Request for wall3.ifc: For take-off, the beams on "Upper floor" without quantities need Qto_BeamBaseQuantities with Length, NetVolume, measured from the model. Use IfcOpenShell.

First a look at what the model holds.

```python
import ifcopenshell
import ifcopenshell.util.element
import ifcopenshell.util.unit

model = ifcopenshell.open("wall3.ifc")
print(model.schema)
for unit_type in ("LENGTHUNIT", "AREAUNIT", "VOLUMEUNIT"):
    print(unit_type, ifcopenshell.util.unit.calculate_unit_scale(model, unit_type))
storey = next(s for s in model.by_type("IfcBuildingStorey") if s.Name == "Upper floor")
beams = [e for e in ifcopenshell.util.element.get_decomposition(storey) if e.is_a("IfcBeam")]
for e in sorted(beams, key=lambda e: e.id()):
    print(e.id(), e.is_a(), e.Name, list(ifcopenshell.util.element.get_psets(e, qtos_only=True)), sep=" | ")
```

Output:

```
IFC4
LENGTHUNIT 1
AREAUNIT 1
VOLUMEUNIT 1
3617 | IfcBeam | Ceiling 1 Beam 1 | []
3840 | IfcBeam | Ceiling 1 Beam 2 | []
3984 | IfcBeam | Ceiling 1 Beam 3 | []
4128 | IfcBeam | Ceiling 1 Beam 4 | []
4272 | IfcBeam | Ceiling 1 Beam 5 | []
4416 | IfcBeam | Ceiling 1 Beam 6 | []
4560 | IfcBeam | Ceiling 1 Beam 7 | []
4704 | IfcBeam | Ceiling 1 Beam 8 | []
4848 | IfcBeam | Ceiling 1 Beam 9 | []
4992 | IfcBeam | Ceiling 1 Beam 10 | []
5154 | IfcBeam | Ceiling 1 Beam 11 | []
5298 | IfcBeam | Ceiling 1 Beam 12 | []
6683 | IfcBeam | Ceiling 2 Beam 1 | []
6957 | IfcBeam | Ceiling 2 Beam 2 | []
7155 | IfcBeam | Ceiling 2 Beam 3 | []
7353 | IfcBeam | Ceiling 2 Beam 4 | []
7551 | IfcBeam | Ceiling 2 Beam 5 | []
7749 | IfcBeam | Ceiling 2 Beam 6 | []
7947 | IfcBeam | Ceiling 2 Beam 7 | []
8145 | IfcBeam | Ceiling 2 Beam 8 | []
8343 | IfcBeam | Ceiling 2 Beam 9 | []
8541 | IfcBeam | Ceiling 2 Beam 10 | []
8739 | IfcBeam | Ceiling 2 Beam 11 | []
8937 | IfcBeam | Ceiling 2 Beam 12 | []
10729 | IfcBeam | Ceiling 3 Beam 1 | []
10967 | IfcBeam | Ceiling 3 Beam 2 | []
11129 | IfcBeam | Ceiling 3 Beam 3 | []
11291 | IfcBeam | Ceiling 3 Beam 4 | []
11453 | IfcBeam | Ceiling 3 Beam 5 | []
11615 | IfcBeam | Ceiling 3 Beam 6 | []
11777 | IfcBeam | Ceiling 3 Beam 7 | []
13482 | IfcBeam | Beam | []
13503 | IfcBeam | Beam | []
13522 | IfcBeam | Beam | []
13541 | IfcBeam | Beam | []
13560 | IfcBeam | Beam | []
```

```python
import ifcopenshell
import ifcopenshell.api.pset
import ifcopenshell.geom
import ifcopenshell.util.element
import ifcopenshell.util.shape
import ifcopenshell.util.unit

model = ifcopenshell.open("wall3.ifc")
unit_scale = ifcopenshell.util.unit.calculate_unit_scale(model)
volume_scale = ifcopenshell.util.unit.calculate_unit_scale(model, "VOLUMEUNIT")
settings = ifcopenshell.geom.settings()

storey = next(s for s in model.by_type("IfcBuildingStorey") if s.Name == "Upper floor")
beams = [e for e in ifcopenshell.util.element.get_decomposition(storey) if e.is_a("IfcBeam")]

for e in sorted(beams, key=lambda e: e.id()):
    if ifcopenshell.util.element.get_psets(e, qtos_only=True, should_inherit=False):
        continue
    # Geometry comes back in metres, in the element's own axes.
    shape = ifcopenshell.geom.create_shape(settings, e)
    values = {
        "Length": ifcopenshell.util.shape.get_max_xyz(shape.geometry) / unit_scale,
        "NetVolume": ifcopenshell.util.shape.get_volume(shape.geometry) / volume_scale,
    }
    qto = ifcopenshell.api.pset.add_qto(model, product=e, name="Qto_BeamBaseQuantities")
    ifcopenshell.api.pset.edit_qto(model, qto=qto, properties=values)
    print(e.id(), {k: round(v, 3) for k, v in values.items()})

model.write("wall3-out.ifc")
```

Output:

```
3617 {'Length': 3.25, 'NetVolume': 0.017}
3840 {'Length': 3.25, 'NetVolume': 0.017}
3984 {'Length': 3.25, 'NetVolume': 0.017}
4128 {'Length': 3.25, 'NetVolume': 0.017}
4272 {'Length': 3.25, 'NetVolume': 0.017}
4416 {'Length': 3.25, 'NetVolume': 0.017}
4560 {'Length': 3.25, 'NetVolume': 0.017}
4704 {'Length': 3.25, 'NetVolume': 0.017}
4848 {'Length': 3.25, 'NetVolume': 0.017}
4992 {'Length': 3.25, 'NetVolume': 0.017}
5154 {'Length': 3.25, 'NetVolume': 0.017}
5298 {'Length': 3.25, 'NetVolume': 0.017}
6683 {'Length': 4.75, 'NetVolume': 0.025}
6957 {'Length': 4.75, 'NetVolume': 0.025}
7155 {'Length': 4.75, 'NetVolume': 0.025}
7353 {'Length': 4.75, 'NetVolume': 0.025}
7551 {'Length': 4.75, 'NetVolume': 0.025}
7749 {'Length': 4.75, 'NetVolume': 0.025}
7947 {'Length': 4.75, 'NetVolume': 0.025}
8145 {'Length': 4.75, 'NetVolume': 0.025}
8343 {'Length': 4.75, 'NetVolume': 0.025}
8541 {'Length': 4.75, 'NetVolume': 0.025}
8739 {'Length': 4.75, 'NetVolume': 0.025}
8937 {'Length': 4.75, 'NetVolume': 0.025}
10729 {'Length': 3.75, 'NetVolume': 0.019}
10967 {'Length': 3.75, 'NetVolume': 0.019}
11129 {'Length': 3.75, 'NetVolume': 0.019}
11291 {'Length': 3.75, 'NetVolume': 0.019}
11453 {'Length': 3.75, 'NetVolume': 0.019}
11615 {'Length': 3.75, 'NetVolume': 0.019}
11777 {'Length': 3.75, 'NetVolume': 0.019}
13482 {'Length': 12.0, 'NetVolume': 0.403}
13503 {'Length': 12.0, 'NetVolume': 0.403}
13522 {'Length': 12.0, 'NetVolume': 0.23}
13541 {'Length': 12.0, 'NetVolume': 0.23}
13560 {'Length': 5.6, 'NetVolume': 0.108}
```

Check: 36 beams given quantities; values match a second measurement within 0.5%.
